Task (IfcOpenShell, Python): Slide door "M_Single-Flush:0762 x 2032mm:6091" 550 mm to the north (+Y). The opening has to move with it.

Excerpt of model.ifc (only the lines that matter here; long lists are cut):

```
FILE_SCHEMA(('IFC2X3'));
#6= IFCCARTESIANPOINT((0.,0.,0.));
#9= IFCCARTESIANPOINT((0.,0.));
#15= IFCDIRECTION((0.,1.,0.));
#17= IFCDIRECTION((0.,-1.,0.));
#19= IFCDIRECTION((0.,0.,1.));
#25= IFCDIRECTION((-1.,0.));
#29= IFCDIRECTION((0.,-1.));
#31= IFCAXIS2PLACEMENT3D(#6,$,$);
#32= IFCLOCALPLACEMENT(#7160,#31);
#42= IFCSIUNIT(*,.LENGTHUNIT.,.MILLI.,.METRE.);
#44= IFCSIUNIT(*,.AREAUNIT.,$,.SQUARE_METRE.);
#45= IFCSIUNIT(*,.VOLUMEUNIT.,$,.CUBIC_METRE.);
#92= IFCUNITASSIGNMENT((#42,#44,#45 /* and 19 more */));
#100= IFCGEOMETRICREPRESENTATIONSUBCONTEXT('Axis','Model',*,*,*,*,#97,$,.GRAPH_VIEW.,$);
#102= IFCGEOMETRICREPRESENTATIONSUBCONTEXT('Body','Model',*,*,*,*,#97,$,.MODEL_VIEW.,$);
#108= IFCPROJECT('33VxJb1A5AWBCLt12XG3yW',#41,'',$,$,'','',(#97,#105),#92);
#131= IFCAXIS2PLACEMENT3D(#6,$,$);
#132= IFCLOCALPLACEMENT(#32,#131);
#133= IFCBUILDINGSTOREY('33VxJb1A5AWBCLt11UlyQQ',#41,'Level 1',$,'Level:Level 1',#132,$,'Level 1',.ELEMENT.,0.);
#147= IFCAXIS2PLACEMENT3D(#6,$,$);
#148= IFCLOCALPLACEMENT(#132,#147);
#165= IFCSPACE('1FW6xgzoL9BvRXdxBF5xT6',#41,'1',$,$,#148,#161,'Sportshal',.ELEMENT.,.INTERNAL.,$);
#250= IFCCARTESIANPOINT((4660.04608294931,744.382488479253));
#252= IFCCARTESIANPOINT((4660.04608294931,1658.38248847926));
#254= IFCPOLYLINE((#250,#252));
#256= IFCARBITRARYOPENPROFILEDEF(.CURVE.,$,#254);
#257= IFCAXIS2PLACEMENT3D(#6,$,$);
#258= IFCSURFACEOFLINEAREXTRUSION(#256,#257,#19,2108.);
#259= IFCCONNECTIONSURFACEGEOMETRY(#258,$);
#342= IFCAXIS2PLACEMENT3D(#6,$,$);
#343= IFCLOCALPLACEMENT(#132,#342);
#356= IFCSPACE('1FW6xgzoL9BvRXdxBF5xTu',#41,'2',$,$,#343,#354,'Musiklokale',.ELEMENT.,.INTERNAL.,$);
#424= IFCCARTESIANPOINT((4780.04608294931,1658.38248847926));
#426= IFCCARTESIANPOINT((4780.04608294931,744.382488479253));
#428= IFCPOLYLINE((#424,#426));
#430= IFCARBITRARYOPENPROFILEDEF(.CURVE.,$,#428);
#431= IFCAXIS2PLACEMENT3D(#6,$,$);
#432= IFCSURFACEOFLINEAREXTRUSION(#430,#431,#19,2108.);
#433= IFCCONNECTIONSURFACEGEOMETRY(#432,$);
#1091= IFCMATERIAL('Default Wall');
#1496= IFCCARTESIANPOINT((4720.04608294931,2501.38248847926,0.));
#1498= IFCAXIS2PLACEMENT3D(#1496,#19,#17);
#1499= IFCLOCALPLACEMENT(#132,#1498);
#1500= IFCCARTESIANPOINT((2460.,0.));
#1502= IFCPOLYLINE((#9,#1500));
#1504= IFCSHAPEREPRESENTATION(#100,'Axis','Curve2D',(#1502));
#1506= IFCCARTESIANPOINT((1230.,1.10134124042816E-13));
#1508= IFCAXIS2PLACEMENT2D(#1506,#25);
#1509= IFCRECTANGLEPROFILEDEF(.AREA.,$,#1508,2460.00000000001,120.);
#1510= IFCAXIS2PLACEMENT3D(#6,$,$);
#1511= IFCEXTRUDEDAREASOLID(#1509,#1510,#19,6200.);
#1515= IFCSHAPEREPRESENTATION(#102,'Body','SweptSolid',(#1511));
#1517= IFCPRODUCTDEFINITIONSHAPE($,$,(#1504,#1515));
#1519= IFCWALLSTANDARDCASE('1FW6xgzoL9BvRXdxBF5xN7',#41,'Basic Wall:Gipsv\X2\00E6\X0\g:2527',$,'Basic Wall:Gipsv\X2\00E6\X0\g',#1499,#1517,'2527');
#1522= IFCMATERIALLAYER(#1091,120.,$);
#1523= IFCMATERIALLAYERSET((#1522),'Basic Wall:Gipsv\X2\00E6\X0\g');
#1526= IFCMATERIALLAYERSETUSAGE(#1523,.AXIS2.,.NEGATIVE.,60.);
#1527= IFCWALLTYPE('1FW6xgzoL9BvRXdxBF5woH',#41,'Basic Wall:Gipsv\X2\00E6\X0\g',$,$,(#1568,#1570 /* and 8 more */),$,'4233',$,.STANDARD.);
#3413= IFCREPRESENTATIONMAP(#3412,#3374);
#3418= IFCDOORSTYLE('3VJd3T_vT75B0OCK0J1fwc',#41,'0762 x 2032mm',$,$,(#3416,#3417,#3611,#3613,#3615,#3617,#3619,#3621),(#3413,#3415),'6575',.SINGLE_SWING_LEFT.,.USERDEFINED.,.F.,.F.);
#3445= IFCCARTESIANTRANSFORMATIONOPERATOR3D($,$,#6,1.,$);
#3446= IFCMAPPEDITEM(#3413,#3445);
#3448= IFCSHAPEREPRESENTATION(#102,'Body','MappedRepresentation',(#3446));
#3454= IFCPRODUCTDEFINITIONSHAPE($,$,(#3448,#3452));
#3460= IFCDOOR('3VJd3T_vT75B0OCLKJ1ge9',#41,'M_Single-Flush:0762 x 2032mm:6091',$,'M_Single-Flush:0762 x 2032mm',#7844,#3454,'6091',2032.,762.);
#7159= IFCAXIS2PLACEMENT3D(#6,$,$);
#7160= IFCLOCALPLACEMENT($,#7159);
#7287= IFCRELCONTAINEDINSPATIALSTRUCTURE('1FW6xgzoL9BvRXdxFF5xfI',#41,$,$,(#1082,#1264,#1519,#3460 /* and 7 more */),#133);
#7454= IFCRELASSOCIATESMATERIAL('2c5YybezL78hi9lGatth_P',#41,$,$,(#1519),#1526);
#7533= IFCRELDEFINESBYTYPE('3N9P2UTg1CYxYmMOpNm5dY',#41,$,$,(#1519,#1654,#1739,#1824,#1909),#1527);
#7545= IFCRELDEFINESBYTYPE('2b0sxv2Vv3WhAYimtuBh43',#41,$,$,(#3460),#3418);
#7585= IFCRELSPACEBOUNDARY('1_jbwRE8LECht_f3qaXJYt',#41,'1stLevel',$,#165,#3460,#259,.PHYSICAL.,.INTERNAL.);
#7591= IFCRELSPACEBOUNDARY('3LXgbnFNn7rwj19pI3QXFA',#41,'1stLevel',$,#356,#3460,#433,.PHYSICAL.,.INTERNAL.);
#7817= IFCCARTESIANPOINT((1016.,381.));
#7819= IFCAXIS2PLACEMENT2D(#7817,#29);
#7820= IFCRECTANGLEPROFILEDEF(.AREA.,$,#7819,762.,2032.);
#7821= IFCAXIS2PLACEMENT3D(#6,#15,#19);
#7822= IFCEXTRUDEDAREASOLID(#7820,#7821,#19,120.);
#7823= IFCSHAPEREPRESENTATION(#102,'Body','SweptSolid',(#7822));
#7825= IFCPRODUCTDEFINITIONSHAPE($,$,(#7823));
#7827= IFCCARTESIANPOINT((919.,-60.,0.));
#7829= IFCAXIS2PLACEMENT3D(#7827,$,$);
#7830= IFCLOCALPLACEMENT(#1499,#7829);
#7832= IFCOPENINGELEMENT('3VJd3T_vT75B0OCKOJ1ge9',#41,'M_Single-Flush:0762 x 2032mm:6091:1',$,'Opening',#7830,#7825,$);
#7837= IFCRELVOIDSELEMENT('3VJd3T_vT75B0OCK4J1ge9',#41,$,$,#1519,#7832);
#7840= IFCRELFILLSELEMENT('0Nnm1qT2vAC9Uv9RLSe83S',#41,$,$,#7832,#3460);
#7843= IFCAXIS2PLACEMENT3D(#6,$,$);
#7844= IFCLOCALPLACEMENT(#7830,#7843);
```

```python
import numpy as np
import ifcopenshell
import ifcopenshell.api.geometry
import ifcopenshell.util.placement

model = ifcopenshell.open("model.ifc")

door = model.by_id(3460)
opening = door.FillsVoids[0].RelatingOpeningElement
wall = opening.VoidsElements[0].RelatingBuildingElement

wall_matrix = ifcopenshell.util.placement.get_local_placement(wall.ObjectPlacement)
shift = wall_matrix[:3, 0] * -550.0
before = ifcopenshell.util.placement.get_local_placement(door.ObjectPlacement)[:3, 3].copy()

# The door is placed relative to its opening, so it follows when the opening moves.
matrix = ifcopenshell.util.placement.get_local_placement(opening.ObjectPlacement)
matrix[:3, 3] += shift
ifcopenshell.api.geometry.edit_object_placement(
    model, product=opening, matrix=matrix, is_si=False, should_transform_children=True
)

# Space boundary surfaces are stored in each space's coordinates; move them too.
for rel in door.ProvidesBoundaries:
    if not rel.ConnectionGeometry:
        continue
    surface = rel.ConnectionGeometry.SurfaceOnRelatingElement
    space_matrix = ifcopenshell.util.placement.get_local_placement(rel.RelatingSpace.ObjectPlacement)
    point = np.array(surface.Position.Location.Coordinates) + space_matrix[:3, :3].T @ shift
    surface.Position = model.createIfcAxis2Placement3D(
        model.createIfcCartesianPoint(point.tolist()), surface.Position.Axis, surface.Position.RefDirection
    )

after = ifcopenshell.util.placement.get_local_placement(door.ObjectPlacement)[:3, 3]
print("door moved by", (after - before).round(3) + 0.0)

model.write("model-out.ifc")
```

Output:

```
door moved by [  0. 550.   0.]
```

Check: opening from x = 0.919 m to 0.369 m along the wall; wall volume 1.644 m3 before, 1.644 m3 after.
